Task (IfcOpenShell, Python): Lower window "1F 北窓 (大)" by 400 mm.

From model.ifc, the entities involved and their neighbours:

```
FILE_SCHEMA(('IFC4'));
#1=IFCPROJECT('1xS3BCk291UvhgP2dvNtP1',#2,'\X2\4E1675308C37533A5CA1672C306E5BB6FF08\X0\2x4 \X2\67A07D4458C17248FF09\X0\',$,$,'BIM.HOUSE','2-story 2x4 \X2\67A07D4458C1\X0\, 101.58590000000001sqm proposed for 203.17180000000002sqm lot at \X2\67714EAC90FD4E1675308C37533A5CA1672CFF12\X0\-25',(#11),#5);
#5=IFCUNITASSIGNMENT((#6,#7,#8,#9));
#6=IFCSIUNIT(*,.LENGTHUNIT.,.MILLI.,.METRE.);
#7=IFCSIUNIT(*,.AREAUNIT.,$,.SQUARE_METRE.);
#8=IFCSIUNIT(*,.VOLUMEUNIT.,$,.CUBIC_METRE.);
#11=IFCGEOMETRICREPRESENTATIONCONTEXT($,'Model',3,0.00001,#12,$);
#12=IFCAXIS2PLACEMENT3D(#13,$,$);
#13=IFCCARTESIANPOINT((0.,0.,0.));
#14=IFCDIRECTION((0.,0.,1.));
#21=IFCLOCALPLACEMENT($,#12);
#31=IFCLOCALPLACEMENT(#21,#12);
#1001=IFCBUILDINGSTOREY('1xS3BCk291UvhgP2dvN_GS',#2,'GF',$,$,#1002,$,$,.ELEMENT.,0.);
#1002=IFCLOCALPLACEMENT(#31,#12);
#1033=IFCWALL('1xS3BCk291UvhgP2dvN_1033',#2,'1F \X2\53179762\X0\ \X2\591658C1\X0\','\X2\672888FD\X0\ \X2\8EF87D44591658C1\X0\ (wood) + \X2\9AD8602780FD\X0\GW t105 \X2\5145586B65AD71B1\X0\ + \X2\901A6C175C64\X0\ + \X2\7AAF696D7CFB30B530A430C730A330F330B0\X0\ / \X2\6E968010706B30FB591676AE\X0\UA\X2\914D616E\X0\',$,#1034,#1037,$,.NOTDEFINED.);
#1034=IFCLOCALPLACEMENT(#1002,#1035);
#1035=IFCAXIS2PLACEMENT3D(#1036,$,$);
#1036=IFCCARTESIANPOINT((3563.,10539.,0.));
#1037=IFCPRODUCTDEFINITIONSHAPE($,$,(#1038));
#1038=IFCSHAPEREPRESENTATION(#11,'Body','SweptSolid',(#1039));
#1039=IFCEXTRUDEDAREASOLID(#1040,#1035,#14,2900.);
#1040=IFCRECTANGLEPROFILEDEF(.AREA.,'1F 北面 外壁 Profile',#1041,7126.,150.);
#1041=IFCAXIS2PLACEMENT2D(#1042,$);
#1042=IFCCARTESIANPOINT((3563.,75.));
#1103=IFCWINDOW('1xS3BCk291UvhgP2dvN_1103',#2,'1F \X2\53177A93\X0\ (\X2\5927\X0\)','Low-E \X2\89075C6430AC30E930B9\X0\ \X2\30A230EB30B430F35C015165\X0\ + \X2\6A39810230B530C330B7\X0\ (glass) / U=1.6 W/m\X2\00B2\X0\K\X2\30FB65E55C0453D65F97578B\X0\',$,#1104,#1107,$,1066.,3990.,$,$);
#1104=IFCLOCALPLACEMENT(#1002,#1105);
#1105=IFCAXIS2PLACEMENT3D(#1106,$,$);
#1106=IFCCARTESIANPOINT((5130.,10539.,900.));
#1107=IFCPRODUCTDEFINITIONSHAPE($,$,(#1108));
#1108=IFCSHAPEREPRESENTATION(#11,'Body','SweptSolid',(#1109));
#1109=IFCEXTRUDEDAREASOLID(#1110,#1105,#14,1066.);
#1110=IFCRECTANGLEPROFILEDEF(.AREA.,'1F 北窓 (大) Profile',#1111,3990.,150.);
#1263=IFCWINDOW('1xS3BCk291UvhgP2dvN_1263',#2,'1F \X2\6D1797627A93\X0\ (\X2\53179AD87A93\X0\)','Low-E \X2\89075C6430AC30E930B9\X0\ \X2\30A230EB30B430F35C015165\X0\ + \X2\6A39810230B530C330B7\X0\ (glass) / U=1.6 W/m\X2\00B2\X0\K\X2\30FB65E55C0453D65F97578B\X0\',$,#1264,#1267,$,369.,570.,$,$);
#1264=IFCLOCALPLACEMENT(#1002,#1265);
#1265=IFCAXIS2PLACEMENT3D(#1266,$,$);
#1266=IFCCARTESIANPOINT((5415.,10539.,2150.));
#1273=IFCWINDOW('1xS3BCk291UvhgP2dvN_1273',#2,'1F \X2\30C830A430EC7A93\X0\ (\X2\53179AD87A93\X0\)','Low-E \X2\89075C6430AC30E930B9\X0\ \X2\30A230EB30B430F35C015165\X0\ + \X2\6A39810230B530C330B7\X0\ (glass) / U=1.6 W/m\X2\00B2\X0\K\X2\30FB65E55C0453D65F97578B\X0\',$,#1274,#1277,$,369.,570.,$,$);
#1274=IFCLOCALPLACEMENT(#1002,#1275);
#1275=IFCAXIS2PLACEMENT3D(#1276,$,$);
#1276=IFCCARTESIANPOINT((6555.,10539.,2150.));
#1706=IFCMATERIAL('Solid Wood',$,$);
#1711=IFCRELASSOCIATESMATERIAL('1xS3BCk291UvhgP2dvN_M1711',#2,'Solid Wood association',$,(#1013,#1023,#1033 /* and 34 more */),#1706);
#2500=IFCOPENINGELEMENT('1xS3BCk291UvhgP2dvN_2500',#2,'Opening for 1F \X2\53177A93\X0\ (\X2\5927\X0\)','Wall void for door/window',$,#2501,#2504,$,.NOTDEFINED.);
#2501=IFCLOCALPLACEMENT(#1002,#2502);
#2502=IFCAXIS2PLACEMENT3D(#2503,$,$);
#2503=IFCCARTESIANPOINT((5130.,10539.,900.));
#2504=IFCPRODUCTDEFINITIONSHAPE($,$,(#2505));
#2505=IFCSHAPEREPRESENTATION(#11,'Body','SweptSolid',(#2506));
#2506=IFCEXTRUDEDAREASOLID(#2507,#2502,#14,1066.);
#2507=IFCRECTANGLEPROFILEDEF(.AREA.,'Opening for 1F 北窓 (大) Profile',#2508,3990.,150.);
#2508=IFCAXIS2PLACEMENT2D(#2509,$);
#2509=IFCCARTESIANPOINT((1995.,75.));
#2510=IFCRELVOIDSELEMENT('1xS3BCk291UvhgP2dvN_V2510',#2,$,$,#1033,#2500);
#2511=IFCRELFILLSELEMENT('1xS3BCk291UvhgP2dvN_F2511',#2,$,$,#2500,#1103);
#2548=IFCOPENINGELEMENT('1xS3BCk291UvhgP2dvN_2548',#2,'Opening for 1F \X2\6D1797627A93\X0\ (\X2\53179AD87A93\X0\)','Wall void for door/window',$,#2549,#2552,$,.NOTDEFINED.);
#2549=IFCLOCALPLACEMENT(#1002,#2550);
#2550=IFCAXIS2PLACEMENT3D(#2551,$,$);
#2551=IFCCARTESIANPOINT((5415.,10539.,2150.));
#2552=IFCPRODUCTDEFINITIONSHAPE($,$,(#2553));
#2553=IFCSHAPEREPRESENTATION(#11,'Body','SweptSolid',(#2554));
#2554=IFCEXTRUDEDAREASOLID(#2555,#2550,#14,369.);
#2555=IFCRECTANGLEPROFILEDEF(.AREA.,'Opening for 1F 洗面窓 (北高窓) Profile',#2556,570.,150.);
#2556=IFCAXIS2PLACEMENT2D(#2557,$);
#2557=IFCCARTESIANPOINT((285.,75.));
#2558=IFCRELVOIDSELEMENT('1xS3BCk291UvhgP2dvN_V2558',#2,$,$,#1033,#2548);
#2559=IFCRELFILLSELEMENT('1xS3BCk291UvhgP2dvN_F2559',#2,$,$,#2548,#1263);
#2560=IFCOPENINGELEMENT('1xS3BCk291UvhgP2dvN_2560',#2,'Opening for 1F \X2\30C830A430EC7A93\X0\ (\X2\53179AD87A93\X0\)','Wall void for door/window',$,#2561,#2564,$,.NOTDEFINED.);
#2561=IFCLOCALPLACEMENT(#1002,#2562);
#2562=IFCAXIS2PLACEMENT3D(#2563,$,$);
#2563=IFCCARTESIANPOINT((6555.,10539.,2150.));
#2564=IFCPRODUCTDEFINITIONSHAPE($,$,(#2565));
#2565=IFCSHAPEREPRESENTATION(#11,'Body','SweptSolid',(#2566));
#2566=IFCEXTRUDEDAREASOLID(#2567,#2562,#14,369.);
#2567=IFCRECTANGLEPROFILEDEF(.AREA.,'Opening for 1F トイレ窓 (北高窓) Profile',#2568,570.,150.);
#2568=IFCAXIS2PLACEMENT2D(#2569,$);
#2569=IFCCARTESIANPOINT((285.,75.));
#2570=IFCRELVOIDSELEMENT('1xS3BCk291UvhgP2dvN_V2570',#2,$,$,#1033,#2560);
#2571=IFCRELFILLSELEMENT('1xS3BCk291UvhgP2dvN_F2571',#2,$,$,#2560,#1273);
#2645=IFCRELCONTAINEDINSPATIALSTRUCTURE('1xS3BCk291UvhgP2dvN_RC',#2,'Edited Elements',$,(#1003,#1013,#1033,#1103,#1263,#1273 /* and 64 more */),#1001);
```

```python
import numpy as np
import ifcopenshell
import ifcopenshell.api.geometry
import ifcopenshell.util.placement
import ifcopenshell.util.unit

model = ifcopenshell.open("model.ifc")
unit_scale = ifcopenshell.util.unit.calculate_unit_scale(model)

window = model.by_id(1103)
opening = window.FillsVoids[0].RelatingOpeningElement
dz = -0.4 / unit_scale

shift = np.array([0.0, 0.0, dz])
# The window is not placed relative to its opening, so move both.
for product in (opening, window):
    matrix = ifcopenshell.util.placement.get_local_placement(product.ObjectPlacement)
    matrix[:3, 3] += shift
    ifcopenshell.api.geometry.edit_object_placement(model, product=product, matrix=matrix, is_si=False)

print(f"moved by {dz * unit_scale:+.3f} m")

model.write("model_updated.ifc")
```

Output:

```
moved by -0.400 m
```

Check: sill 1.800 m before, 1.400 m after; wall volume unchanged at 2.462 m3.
